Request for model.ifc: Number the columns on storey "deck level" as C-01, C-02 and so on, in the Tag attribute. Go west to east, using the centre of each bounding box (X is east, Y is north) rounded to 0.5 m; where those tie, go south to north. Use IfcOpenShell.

First a look at what the model holds.

```python
import ifcopenshell
import ifcopenshell.util.element
import ifcopenshell.util.placement

model = ifcopenshell.open("model.ifc")
print(model.schema)
storey = next(s for s in model.by_type("IfcBuildingStorey") if s.Name == "deck level")
columns = [e for e in ifcopenshell.util.element.get_decomposition(storey) if e.is_a("IfcColumn")]
for e in sorted(columns, key=lambda e: e.id()):
    origin = ifcopenshell.util.placement.get_local_placement(e.ObjectPlacement)[:3, 3]
    print(e.id(), e.Tag, e.Name, origin.round(2) + 0.0, sep=" | ")
```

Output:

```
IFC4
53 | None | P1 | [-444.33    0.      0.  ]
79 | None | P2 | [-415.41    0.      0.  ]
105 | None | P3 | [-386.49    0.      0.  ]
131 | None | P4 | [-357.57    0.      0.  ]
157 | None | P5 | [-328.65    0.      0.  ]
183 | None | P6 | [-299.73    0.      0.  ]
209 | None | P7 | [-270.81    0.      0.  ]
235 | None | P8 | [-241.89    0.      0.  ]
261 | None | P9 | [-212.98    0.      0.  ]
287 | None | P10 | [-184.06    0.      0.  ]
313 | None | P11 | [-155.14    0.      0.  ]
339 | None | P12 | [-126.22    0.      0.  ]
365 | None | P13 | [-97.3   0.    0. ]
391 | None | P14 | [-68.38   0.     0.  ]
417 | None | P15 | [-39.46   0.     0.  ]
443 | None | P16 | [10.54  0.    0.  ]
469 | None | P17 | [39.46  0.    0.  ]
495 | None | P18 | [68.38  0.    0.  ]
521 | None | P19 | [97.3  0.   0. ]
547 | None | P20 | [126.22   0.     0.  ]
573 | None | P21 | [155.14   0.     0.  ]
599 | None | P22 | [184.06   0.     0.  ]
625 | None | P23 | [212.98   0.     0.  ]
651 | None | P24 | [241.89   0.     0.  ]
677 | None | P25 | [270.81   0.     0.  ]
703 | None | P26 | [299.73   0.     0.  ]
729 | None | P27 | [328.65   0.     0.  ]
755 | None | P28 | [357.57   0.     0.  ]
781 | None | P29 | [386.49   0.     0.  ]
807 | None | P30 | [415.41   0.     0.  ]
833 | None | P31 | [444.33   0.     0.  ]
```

```python
import ifcopenshell
import ifcopenshell.geom
import ifcopenshell.util.element
import ifcopenshell.util.shape

model = ifcopenshell.open("model.ifc")
settings = ifcopenshell.geom.settings()
settings.set("use-world-coords", True)


def centre(element):
    shape = ifcopenshell.geom.create_shape(settings, element)
    return ifcopenshell.util.shape.get_bbox_centroid(shape.geometry)


storey = next(s for s in model.by_type("IfcBuildingStorey") if s.Name == "deck level")
columns = [e for e in ifcopenshell.util.element.get_decomposition(storey) if e.is_a("IfcColumn")]

# Insertion points can sit at a corner or the storey origin, so sort by the geometry (in metres).
centres = {e: centre(e) for e in columns}
columns.sort(key=lambda e: (round(centres[e][0] / 0.5), centres[e][1]))

for i, e in enumerate(columns, start=1):
    number = f"C-{i:02d}"
    e.Tag = number
    print(e.id(), number)

model.write("model_v2.ifc")
```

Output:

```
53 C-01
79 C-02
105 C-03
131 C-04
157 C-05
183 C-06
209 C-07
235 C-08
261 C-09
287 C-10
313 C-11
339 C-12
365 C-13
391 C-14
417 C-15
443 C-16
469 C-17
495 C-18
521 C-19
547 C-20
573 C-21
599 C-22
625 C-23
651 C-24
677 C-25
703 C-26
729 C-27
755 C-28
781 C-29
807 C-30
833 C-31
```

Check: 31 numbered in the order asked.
